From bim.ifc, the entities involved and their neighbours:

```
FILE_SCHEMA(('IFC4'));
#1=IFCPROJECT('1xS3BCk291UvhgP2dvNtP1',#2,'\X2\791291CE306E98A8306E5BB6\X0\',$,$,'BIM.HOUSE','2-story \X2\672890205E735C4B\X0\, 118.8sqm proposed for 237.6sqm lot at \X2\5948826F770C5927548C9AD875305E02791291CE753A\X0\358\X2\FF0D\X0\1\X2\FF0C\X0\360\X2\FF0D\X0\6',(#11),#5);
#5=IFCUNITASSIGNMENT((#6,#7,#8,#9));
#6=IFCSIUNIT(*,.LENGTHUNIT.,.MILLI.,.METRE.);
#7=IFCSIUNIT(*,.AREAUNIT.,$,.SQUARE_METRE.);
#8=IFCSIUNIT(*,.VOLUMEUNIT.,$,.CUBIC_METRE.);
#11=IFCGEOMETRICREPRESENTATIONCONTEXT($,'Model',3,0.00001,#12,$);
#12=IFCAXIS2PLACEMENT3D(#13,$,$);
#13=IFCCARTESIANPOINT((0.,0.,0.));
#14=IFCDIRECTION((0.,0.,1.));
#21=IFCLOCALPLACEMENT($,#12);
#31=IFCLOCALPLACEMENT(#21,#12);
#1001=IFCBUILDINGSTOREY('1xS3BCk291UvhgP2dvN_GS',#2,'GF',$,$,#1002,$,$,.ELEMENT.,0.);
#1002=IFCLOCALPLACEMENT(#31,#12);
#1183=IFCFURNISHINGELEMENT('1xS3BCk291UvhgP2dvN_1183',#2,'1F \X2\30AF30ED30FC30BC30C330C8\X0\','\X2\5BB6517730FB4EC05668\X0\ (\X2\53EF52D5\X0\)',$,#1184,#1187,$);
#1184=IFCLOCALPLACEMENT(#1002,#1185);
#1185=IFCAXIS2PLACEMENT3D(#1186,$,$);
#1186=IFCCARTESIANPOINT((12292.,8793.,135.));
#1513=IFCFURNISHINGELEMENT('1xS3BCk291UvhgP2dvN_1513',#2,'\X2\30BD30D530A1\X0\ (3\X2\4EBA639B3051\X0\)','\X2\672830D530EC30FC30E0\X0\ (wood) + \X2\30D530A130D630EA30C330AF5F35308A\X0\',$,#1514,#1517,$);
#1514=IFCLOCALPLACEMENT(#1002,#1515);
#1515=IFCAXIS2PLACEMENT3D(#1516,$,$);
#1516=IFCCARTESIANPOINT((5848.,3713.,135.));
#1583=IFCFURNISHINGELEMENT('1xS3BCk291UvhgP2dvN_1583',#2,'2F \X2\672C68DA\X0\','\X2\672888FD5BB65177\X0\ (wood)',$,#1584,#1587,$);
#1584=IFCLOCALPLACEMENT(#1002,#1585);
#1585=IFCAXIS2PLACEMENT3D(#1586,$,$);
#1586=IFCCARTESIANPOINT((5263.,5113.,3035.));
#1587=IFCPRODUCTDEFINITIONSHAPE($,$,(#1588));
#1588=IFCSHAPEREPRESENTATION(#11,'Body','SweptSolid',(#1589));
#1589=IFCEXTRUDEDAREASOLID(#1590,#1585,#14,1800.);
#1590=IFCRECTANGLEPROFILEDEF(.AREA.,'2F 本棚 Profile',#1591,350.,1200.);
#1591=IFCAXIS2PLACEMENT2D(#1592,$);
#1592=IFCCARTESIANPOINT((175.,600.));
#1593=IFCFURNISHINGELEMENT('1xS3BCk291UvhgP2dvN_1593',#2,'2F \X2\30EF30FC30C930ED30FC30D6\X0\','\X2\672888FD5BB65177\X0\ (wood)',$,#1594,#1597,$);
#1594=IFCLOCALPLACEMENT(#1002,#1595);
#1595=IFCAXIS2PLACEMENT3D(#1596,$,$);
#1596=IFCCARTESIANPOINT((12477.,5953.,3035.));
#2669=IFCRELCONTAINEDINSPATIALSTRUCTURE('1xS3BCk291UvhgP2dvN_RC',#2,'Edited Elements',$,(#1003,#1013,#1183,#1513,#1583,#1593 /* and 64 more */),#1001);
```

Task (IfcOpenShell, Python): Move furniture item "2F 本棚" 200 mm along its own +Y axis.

```python
import ifcopenshell
import ifcopenshell.api.geometry
import ifcopenshell.util.placement
import ifcopenshell.util.unit

model = ifcopenshell.open("bim.ifc")
unit_scale = ifcopenshell.util.unit.calculate_unit_scale(model)

item = model.by_guid("1xS3BCk291UvhgP2dvN_1583")
matrix = ifcopenshell.util.placement.get_local_placement(item.ObjectPlacement)
matrix[:3, 3] += matrix[:3, 1] * 0.2 / unit_scale
ifcopenshell.api.geometry.edit_object_placement(model, product=item, matrix=matrix, is_si=False)

print(ifcopenshell.util.placement.get_local_placement(item.ObjectPlacement).round(3) + 0.0)

model.write("bim-out.ifc")
```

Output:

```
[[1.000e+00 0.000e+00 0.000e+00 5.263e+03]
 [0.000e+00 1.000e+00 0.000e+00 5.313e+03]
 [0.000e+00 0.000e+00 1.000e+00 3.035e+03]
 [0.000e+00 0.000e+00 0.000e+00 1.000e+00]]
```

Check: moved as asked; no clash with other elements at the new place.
